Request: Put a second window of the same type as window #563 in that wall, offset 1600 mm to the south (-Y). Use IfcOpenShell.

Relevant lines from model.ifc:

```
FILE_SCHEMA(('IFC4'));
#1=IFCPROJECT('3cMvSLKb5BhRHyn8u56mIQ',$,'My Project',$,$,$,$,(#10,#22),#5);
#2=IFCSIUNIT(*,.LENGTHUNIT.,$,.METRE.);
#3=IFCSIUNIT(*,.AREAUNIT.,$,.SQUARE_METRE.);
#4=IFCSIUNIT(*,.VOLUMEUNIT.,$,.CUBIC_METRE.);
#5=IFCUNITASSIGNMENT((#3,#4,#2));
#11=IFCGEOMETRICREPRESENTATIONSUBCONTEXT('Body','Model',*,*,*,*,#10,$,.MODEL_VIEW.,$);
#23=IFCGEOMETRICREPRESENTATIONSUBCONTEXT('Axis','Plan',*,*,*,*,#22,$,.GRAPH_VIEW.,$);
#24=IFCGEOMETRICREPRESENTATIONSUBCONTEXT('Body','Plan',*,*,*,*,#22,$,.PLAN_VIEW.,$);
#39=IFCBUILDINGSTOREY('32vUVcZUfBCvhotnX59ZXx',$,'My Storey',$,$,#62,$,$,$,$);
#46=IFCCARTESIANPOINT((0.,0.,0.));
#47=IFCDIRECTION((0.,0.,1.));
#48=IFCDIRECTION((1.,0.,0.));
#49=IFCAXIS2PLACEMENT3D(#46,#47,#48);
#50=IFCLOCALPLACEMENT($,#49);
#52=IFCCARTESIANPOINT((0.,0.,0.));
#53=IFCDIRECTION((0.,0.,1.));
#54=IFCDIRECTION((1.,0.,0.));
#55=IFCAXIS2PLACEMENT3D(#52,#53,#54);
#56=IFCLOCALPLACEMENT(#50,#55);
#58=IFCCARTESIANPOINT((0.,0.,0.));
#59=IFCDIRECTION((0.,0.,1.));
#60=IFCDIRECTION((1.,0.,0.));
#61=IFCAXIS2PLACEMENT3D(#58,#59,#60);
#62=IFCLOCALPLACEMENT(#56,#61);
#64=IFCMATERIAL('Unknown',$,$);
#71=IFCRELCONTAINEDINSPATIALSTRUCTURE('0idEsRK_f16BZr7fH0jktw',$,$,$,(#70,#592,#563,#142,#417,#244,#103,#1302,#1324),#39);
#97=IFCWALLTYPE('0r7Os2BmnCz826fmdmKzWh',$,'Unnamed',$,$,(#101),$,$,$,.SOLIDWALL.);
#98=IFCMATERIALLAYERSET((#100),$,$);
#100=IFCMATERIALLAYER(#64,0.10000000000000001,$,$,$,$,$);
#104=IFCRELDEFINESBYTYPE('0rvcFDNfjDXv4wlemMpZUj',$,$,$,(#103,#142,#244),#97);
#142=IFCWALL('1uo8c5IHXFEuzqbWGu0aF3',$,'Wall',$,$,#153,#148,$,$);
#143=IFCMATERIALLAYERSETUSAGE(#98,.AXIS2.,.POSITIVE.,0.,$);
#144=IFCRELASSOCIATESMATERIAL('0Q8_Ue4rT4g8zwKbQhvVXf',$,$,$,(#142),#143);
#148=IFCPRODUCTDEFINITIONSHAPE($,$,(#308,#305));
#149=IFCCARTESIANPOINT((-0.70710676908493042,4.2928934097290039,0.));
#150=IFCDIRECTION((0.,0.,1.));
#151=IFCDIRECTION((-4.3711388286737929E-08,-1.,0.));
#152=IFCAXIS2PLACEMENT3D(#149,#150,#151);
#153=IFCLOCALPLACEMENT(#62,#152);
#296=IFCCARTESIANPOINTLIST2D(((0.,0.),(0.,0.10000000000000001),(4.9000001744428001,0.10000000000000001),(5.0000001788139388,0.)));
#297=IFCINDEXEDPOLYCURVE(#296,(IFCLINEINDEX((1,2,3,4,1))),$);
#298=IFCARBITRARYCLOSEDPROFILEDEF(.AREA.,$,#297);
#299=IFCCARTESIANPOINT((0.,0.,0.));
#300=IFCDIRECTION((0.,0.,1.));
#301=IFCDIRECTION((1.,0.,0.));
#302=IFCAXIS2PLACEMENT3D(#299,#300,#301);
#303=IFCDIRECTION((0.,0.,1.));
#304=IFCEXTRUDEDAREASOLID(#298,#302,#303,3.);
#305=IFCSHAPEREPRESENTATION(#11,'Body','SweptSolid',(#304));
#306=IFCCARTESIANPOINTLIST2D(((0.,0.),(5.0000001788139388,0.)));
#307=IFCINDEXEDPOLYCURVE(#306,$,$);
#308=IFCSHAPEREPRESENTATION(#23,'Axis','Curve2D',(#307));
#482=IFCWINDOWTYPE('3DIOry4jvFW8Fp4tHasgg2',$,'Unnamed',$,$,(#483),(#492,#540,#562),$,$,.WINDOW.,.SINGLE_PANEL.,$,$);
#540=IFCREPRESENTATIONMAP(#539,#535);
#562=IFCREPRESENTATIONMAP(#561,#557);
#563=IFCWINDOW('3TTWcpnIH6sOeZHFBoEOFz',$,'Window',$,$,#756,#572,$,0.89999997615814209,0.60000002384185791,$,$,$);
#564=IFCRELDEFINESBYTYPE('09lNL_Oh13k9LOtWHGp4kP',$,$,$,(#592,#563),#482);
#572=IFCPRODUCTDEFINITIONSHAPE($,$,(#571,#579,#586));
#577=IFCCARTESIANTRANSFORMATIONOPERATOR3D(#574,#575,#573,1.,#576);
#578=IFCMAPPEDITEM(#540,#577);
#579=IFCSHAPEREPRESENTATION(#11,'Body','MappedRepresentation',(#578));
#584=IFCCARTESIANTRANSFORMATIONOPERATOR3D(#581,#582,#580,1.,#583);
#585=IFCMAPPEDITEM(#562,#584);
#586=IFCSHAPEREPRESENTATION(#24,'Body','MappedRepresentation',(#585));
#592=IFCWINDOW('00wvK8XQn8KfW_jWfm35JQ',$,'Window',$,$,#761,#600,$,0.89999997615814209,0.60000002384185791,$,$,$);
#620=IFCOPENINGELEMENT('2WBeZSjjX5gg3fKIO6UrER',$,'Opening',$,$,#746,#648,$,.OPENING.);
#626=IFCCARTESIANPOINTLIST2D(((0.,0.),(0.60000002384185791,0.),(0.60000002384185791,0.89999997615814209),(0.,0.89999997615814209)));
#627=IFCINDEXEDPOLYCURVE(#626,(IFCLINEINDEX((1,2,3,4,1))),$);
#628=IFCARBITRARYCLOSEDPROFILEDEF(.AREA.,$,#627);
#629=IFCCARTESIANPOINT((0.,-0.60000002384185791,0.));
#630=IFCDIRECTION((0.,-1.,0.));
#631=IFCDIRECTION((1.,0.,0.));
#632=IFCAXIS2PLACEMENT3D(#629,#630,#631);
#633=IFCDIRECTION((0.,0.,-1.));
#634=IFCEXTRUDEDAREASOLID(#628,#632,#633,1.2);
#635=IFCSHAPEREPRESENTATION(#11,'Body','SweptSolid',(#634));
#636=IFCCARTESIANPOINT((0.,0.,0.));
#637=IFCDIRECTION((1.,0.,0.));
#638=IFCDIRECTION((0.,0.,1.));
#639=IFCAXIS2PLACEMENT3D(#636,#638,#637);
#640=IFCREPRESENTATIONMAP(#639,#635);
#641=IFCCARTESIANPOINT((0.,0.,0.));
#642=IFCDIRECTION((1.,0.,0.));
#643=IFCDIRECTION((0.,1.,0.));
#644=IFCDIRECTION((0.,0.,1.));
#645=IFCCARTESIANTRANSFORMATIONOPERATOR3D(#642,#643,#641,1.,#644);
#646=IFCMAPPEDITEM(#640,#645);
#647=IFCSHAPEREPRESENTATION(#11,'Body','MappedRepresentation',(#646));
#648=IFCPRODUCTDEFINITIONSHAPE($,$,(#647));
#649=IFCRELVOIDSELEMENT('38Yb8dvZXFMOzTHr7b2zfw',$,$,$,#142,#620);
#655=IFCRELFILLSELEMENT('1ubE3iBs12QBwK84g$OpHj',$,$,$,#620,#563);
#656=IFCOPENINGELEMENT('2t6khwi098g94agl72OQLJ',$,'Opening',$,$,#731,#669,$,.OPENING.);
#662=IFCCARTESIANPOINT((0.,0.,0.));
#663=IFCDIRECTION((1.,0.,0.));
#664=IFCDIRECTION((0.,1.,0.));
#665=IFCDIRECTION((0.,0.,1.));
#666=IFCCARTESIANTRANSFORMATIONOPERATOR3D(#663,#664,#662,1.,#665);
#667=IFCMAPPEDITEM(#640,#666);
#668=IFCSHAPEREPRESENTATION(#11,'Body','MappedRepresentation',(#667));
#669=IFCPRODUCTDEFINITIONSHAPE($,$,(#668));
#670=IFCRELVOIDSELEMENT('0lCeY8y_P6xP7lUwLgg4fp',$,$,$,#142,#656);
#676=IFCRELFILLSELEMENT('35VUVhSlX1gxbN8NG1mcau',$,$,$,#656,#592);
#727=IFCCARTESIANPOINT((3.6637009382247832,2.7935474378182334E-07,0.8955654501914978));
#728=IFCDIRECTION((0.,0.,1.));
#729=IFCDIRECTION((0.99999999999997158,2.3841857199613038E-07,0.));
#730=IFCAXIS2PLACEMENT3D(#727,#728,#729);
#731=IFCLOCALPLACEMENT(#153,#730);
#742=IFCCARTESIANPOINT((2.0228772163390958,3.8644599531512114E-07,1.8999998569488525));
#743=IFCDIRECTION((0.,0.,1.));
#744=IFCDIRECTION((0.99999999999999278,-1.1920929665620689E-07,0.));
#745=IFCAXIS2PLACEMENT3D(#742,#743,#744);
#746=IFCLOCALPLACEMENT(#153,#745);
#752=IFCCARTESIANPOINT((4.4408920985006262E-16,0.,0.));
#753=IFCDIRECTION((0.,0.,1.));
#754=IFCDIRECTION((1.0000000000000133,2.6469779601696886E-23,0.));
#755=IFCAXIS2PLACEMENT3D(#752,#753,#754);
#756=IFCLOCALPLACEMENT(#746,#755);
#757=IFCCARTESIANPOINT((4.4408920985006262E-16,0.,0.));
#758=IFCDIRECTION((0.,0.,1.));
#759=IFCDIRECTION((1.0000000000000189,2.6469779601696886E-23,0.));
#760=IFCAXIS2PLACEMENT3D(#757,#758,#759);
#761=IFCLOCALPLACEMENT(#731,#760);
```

```python
import ifcopenshell
import ifcopenshell.api.feature
import ifcopenshell.api.geometry
import ifcopenshell.api.root
import ifcopenshell.geom
import ifcopenshell.util.element
import ifcopenshell.util.placement
import ifcopenshell.util.shape
import ifcopenshell.util.unit

model = ifcopenshell.open("model.ifc")
unit_scale = ifcopenshell.util.unit.calculate_unit_scale(model)
settings = ifcopenshell.geom.settings()


def volume(element):
    """Net volume in cubic metres, openings subtracted."""
    shape = ifcopenshell.geom.create_shape(settings, element)
    return ifcopenshell.util.shape.get_volume(shape.geometry)


window = model.by_guid("3TTWcpnIH6sOeZHFBoEOFz")
opening = window.FillsVoids[0].RelatingOpeningElement
wall = opening.VoidsElements[0].RelatingBuildingElement
before = volume(wall)
shift = ifcopenshell.util.placement.get_local_placement(wall.ObjectPlacement)[:3, 0] * 1.6 / unit_scale

# copy_class copies the void relationship, type, container and properties, but no geometry.
new_opening = ifcopenshell.api.root.copy_class(model, product=opening)
new_opening.Representation = ifcopenshell.util.element.copy_deep(
    model, opening.Representation, exclude=["IfcGeometricRepresentationContext", "IfcRepresentationMap"]
)
new_window = ifcopenshell.api.root.copy_class(model, product=window)
new_window.Representation = ifcopenshell.util.element.copy_deep(
    model, window.Representation, exclude=["IfcGeometricRepresentationContext", "IfcRepresentationMap"]
)
ifcopenshell.api.feature.add_filling(model, opening=new_opening, element=new_window)

for old, new in ((opening, new_opening), (window, new_window)):
    matrix = ifcopenshell.util.placement.get_local_placement(old.ObjectPlacement)
    matrix[:3, 3] += shift
    ifcopenshell.api.geometry.edit_object_placement(model, product=new, matrix=matrix, is_si=False)

after = volume(wall)

print(f"wall volume {before:.3f} -> {after:.3f} m3")

model.write("model_v2.ifc")
```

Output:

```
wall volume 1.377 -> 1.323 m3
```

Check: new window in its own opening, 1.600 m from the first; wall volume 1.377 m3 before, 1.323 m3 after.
